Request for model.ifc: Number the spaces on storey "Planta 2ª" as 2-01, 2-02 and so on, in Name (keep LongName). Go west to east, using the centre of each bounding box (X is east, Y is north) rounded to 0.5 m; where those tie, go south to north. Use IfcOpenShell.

First a look at what the model holds.

```python
import ifcopenshell
import ifcopenshell.util.element
import ifcopenshell.util.placement

model = ifcopenshell.open("model.ifc")
print(model.schema)
storey = next(s for s in model.by_type("IfcBuildingStorey") if s.Name == "Planta 2ª")
spaces = [e for e in ifcopenshell.util.element.get_decomposition(storey) if e.is_a("IfcSpace")]
for e in sorted(spaces, key=lambda e: e.id()):
    origin = ifcopenshell.util.placement.get_local_placement(e.ObjectPlacement)[:3, 3]
    print(e.id(), e.Name, e.LongName, origin.round(2) + 0.0, sep=" | ")
```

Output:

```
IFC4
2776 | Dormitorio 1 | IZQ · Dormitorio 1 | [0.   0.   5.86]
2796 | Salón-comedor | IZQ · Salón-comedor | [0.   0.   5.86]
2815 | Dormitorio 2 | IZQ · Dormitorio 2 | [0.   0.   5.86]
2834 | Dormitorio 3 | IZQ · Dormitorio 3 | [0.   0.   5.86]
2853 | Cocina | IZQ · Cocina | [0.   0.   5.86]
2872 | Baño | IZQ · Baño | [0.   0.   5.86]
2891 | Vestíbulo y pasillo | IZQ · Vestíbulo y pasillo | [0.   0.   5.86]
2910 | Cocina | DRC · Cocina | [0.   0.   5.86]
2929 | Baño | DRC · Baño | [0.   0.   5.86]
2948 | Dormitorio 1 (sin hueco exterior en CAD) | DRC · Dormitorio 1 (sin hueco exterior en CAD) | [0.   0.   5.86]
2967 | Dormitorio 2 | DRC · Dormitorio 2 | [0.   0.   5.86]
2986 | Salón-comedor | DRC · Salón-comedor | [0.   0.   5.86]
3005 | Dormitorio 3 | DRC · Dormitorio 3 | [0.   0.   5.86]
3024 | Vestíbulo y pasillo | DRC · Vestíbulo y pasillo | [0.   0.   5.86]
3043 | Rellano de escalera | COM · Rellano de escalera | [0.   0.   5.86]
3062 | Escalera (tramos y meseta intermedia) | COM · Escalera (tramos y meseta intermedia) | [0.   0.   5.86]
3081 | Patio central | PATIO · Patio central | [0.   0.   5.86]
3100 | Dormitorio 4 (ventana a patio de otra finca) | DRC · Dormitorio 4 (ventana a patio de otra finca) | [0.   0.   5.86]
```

```python
import ifcopenshell
import ifcopenshell.geom
import ifcopenshell.util.element
import ifcopenshell.util.shape

model = ifcopenshell.open("model.ifc")
settings = ifcopenshell.geom.settings()
settings.set("use-world-coords", True)


def centre(element):
    shape = ifcopenshell.geom.create_shape(settings, element)
    return ifcopenshell.util.shape.get_bbox_centroid(shape.geometry)


storey = next(s for s in model.by_type("IfcBuildingStorey") if s.Name == "Planta 2ª")
spaces = [e for e in ifcopenshell.util.element.get_decomposition(storey) if e.is_a("IfcSpace")]

# Insertion points can sit at a corner or the storey origin, so sort by the geometry (in metres).
centres = {e: centre(e) for e in spaces}
spaces.sort(key=lambda e: (round(centres[e][0] / 0.5), centres[e][1]))

for i, e in enumerate(spaces, start=1):
    number = f"2-{i:02d}"
    e.Name = number
    print(e.id(), number)

model.write("model_edited.ifc")
```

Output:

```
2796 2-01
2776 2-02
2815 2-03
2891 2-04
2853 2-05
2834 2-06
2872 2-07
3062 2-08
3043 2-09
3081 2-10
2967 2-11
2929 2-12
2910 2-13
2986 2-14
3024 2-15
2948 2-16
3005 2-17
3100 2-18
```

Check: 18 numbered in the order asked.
